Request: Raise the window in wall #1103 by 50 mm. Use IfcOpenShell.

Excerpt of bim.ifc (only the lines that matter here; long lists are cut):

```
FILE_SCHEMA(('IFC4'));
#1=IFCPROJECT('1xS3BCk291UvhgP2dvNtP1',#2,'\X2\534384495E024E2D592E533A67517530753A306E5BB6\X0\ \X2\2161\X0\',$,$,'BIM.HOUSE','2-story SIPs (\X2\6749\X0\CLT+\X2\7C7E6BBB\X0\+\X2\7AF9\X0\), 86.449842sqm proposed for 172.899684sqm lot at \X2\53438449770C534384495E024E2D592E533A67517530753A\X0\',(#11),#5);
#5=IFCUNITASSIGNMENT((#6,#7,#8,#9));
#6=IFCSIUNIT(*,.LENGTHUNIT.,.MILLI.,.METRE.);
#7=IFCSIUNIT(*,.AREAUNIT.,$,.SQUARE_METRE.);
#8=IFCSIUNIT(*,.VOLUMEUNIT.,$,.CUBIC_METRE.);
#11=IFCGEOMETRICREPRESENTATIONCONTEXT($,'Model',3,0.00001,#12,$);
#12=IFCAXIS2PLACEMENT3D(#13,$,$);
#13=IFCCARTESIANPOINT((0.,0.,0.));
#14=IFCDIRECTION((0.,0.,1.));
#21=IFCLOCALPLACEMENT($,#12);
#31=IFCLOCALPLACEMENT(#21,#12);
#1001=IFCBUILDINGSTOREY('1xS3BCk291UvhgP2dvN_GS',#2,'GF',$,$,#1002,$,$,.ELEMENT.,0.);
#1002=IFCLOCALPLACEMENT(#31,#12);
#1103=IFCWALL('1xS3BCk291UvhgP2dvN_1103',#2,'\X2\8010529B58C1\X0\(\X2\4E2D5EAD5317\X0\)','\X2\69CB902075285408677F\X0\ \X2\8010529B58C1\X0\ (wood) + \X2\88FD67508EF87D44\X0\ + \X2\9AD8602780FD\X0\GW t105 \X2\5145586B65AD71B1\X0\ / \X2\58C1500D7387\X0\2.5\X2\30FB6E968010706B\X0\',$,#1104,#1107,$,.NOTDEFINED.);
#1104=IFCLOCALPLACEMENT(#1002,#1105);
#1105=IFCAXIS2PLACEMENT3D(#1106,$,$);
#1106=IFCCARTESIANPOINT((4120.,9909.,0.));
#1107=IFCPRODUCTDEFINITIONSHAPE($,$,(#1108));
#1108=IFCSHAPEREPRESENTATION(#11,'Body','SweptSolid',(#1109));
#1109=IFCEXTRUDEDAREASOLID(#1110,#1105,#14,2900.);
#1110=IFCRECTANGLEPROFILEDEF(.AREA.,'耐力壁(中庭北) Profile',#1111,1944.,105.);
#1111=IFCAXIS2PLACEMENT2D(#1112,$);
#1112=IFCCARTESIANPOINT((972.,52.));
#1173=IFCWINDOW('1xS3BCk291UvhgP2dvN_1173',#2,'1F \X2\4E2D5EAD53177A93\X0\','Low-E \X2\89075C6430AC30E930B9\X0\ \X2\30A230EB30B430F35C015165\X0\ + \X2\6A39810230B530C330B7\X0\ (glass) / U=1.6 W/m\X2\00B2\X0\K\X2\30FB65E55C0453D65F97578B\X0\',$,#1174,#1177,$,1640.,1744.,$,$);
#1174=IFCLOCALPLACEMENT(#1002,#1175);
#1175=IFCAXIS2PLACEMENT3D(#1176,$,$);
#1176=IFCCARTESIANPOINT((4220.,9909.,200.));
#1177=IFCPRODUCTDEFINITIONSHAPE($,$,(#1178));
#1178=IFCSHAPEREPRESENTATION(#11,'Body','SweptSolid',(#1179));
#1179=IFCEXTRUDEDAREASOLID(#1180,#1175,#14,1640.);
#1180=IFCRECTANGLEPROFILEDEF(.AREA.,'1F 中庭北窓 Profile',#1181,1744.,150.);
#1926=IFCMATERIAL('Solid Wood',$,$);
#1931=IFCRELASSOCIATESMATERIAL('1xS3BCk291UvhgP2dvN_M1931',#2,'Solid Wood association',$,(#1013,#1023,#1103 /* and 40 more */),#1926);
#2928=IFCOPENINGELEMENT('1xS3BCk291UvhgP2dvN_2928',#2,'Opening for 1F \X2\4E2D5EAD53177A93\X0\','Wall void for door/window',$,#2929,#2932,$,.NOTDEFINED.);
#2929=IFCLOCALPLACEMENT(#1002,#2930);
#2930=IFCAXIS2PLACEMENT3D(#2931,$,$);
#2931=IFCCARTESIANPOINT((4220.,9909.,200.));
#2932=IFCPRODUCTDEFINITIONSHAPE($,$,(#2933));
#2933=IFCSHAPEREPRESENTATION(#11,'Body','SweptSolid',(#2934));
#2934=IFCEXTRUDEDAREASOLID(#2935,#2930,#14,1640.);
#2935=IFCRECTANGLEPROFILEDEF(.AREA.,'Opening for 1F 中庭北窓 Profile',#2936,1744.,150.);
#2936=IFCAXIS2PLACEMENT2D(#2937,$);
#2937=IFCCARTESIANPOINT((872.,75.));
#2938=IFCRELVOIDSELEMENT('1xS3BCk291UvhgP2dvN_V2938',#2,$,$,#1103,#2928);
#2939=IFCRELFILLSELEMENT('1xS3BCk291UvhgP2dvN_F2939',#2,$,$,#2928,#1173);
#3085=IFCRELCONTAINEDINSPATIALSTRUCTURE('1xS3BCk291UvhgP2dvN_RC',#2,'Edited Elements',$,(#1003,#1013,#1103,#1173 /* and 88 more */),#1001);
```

```python
import numpy as np
import ifcopenshell
import ifcopenshell.api.geometry
import ifcopenshell.util.placement
import ifcopenshell.util.unit

model = ifcopenshell.open("bim.ifc")
unit_scale = ifcopenshell.util.unit.calculate_unit_scale(model)

window = model.by_guid("1xS3BCk291UvhgP2dvN_1173")
opening = window.FillsVoids[0].RelatingOpeningElement
dz = 0.05 / unit_scale

shift = np.array([0.0, 0.0, dz])
# The window is not placed relative to its opening, so move both.
for product in (opening, window):
    matrix = ifcopenshell.util.placement.get_local_placement(product.ObjectPlacement)
    matrix[:3, 3] += shift
    ifcopenshell.api.geometry.edit_object_placement(model, product=product, matrix=matrix, is_si=False)

print(f"moved by {dz * unit_scale:+.3f} m")

model.write("bim-out.ifc")
```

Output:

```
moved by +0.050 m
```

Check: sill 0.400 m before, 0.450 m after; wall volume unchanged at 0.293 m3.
